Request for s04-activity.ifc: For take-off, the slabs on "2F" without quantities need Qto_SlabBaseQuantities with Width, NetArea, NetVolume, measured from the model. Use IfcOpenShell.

First a look at what the model holds.

```python
import ifcopenshell
import ifcopenshell.util.element
import ifcopenshell.util.unit

model = ifcopenshell.open("s04-activity.ifc")
print(model.schema)
for unit_type in ("LENGTHUNIT", "AREAUNIT", "VOLUMEUNIT"):
    print(unit_type, ifcopenshell.util.unit.calculate_unit_scale(model, unit_type))
storey = next(s for s in model.by_type("IfcBuildingStorey") if s.Name == "2F")
slabs = [e for e in ifcopenshell.util.element.get_decomposition(storey) if e.is_a("IfcSlab")]
for e in sorted(slabs, key=lambda e: e.id()):
    print(e.id(), e.is_a(), e.Name, list(ifcopenshell.util.element.get_psets(e, qtos_only=True)), sep=" | ")
```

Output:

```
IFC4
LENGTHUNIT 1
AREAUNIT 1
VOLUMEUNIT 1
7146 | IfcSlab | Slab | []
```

```python
import ifcopenshell
import ifcopenshell.api.pset
import ifcopenshell.geom
import ifcopenshell.util.element
import ifcopenshell.util.shape
import ifcopenshell.util.unit

model = ifcopenshell.open("s04-activity.ifc")
unit_scale = ifcopenshell.util.unit.calculate_unit_scale(model)
area_scale = ifcopenshell.util.unit.calculate_unit_scale(model, "AREAUNIT")
volume_scale = ifcopenshell.util.unit.calculate_unit_scale(model, "VOLUMEUNIT")
settings = ifcopenshell.geom.settings()

storey = next(s for s in model.by_type("IfcBuildingStorey") if s.Name == "2F")
slabs = [e for e in ifcopenshell.util.element.get_decomposition(storey) if e.is_a("IfcSlab")]

for e in sorted(slabs, key=lambda e: e.id()):
    if ifcopenshell.util.element.get_psets(e, qtos_only=True, should_inherit=False):
        continue
    # Geometry comes back in metres, in the element's own axes.
    shape = ifcopenshell.geom.create_shape(settings, e)
    values = {
        "Width": ifcopenshell.util.shape.get_z(shape.geometry) / unit_scale,
        "NetArea": ifcopenshell.util.shape.get_footprint_area(shape.geometry) / area_scale,
        "NetVolume": ifcopenshell.util.shape.get_volume(shape.geometry) / volume_scale,
    }
    qto = ifcopenshell.api.pset.add_qto(model, product=e, name="Qto_SlabBaseQuantities")
    ifcopenshell.api.pset.edit_qto(model, qto=qto, properties=values)
    print(e.id(), {k: round(v, 3) for k, v in values.items()})

model.write("s04-activity_rev.ifc")
```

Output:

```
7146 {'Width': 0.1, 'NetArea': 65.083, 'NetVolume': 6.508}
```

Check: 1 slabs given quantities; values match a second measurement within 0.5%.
